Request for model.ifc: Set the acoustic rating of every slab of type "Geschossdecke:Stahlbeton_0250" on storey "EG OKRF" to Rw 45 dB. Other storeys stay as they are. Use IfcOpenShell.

First a look at what the model holds.

```python
import ifcopenshell
import ifcopenshell.util.element

model = ifcopenshell.open("model.ifc")
print(model.schema)
storey = next(s for s in model.by_type("IfcBuildingStorey") if s.Name == "EG OKRF")
slabs = [e for e in ifcopenshell.util.element.get_decomposition(storey) if e.is_a("IfcSlab")]
seen = {}
for e in slabs:
    element_type = ifcopenshell.util.element.get_type(e)
    key = (element_type.Name if element_type != e and element_type else None, ifcopenshell.util.element.get_pset(e, "Pset_SlabCommon", "AcousticRating"))
    seen[key] = seen.get(key, 0) + 1
for (name, value), count in sorted(seen.items(), key=str):
    print(count, "x", name, "|", value)
```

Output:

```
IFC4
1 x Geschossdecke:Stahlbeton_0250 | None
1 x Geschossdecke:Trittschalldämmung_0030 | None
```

```python
import ifcopenshell
import ifcopenshell.api.pset
import ifcopenshell.util.element

model = ifcopenshell.open("model.ifc")

storey = next(s for s in model.by_type("IfcBuildingStorey") if s.Name == "EG OKRF")
slabs = [e for e in ifcopenshell.util.element.get_decomposition(storey) if e.is_a("IfcSlab")]

count = 0
for e in slabs:
    element_type = ifcopenshell.util.element.get_type(e)
    if element_type in (None, e) or element_type.Name != "Geschossdecke:Stahlbeton_0250":
        continue
    # add_pset returns the element's existing set when there is one.
    pset = ifcopenshell.api.pset.add_pset(model, product=e, name="Pset_SlabCommon")
    ifcopenshell.api.pset.edit_pset(model, pset=pset, properties={"AcousticRating": "Rw 45 dB"})
    count += 1

print(count, "slabs updated")

model.write("model_v2.ifc")
```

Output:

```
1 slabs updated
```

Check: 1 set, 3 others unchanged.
